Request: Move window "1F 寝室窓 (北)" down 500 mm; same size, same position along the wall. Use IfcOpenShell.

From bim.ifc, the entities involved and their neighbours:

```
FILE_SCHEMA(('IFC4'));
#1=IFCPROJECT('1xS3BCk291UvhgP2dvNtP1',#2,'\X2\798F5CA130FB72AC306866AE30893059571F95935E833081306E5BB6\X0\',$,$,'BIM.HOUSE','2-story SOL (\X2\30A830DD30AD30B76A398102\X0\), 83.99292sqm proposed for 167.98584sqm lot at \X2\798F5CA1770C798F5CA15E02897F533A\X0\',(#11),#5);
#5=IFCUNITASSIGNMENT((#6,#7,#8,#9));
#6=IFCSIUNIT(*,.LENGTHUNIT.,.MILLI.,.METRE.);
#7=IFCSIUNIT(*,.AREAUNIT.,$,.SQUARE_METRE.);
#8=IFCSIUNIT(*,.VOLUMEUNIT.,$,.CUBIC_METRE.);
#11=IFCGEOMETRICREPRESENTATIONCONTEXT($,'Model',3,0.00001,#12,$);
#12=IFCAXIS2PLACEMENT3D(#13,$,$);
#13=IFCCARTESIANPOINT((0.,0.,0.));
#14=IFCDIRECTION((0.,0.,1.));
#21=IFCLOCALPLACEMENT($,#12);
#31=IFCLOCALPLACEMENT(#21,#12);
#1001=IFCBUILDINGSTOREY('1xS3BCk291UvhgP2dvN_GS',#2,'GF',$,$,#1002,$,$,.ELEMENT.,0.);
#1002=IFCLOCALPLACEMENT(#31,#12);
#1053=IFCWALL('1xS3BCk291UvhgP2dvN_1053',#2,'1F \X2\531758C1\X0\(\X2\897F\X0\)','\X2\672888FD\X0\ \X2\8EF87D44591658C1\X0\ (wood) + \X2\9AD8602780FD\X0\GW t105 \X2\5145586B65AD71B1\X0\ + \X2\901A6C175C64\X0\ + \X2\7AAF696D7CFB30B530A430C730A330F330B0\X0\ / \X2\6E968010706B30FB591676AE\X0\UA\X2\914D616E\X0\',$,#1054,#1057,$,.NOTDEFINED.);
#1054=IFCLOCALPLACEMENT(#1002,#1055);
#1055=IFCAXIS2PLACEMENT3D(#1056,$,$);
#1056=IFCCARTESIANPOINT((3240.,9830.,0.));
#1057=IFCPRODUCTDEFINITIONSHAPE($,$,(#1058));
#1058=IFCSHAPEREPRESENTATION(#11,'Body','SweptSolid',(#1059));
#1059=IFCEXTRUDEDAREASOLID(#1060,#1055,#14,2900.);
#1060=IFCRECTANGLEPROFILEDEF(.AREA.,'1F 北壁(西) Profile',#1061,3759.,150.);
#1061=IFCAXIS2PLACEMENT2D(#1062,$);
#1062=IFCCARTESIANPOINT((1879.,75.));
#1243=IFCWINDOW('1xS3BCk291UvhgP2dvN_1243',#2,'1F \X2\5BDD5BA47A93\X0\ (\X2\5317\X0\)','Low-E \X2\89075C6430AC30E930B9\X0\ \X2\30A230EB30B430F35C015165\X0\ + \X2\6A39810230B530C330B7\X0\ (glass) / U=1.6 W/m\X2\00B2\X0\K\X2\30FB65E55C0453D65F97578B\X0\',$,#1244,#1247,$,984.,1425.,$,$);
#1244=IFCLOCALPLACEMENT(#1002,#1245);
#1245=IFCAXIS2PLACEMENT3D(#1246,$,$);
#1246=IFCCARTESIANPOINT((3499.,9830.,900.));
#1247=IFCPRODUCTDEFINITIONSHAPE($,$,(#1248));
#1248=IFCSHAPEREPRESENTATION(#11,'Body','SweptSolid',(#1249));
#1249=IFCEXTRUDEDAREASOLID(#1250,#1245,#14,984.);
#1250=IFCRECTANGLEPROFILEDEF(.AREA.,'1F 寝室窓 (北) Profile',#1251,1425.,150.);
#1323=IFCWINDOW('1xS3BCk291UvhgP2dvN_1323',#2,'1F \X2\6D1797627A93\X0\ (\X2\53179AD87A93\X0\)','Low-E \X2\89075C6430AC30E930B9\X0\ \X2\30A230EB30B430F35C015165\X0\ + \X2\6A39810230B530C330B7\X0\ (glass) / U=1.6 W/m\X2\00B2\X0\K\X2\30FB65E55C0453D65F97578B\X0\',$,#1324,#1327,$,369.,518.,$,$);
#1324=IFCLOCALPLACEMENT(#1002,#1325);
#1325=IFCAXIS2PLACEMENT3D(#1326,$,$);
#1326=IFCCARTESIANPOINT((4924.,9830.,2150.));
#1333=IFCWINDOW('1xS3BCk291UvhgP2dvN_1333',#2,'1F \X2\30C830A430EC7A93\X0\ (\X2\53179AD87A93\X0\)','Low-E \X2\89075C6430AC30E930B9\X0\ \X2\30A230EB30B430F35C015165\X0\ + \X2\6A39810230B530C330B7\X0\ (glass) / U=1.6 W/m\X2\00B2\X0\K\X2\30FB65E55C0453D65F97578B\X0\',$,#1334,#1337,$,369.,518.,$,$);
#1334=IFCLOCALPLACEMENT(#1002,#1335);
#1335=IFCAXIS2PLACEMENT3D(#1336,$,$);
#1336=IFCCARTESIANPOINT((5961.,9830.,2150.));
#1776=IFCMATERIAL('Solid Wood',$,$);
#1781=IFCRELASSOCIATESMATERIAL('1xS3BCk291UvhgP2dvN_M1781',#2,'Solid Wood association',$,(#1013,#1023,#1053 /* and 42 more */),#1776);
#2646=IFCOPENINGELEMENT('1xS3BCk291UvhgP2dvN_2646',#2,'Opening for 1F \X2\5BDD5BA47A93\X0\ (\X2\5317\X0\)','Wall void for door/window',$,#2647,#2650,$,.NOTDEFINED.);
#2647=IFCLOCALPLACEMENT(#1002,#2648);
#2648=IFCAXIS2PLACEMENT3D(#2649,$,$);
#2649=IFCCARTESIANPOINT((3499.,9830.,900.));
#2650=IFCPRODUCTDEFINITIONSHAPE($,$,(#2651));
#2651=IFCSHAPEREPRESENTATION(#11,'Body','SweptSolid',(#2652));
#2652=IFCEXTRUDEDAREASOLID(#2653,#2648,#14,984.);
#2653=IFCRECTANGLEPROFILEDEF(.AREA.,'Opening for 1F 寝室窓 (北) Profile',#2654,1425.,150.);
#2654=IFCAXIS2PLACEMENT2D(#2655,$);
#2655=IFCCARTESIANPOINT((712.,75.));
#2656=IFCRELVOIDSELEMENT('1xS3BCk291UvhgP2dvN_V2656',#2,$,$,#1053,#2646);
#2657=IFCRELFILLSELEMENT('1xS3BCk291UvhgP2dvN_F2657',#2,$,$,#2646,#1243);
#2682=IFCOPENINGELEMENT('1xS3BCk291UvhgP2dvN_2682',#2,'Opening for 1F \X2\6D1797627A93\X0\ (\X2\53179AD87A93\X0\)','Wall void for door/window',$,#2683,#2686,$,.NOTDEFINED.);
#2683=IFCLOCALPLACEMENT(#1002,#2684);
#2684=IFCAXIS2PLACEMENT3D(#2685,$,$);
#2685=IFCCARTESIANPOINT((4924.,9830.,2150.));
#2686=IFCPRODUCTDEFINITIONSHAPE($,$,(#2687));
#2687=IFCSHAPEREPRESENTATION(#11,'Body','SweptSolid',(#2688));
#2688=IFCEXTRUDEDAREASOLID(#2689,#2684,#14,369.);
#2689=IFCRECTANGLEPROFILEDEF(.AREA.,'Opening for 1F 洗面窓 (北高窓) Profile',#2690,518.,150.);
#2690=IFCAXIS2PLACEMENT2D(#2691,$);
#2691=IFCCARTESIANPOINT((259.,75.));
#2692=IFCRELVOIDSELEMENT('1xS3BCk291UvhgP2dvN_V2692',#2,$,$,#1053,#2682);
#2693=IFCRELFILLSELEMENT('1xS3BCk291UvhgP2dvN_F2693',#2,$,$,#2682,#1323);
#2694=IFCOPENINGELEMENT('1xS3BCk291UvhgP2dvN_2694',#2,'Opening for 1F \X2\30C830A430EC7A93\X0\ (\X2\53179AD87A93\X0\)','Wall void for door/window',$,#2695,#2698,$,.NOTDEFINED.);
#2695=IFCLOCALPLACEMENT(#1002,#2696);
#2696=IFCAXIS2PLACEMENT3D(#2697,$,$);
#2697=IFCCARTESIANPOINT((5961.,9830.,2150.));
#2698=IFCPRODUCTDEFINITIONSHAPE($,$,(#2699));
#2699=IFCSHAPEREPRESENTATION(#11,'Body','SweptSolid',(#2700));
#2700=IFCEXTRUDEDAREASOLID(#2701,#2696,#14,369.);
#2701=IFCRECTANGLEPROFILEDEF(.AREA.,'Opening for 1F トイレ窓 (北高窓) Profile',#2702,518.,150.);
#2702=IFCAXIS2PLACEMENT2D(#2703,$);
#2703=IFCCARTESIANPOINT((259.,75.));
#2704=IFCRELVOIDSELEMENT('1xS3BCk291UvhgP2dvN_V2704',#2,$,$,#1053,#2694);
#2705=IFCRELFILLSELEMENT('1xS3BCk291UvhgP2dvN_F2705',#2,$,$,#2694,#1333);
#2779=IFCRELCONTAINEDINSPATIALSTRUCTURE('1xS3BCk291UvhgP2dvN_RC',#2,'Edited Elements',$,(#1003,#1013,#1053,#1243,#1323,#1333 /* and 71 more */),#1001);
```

```python
import numpy as np
import ifcopenshell
import ifcopenshell.api.geometry
import ifcopenshell.util.placement
import ifcopenshell.util.unit

model = ifcopenshell.open("bim.ifc")
unit_scale = ifcopenshell.util.unit.calculate_unit_scale(model)

window = model.by_guid("1xS3BCk291UvhgP2dvN_1243")
opening = window.FillsVoids[0].RelatingOpeningElement
dz = -0.5 / unit_scale

shift = np.array([0.0, 0.0, dz])
# The window is not placed relative to its opening, so move both.
for product in (opening, window):
    matrix = ifcopenshell.util.placement.get_local_placement(product.ObjectPlacement)
    matrix[:3, 3] += shift
    ifcopenshell.api.geometry.edit_object_placement(model, product=product, matrix=matrix, is_si=False)

print(f"moved by {dz * unit_scale:+.3f} m")

model.write("bim_edited.ifc")
```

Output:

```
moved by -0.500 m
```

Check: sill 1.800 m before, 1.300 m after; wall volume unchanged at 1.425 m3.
